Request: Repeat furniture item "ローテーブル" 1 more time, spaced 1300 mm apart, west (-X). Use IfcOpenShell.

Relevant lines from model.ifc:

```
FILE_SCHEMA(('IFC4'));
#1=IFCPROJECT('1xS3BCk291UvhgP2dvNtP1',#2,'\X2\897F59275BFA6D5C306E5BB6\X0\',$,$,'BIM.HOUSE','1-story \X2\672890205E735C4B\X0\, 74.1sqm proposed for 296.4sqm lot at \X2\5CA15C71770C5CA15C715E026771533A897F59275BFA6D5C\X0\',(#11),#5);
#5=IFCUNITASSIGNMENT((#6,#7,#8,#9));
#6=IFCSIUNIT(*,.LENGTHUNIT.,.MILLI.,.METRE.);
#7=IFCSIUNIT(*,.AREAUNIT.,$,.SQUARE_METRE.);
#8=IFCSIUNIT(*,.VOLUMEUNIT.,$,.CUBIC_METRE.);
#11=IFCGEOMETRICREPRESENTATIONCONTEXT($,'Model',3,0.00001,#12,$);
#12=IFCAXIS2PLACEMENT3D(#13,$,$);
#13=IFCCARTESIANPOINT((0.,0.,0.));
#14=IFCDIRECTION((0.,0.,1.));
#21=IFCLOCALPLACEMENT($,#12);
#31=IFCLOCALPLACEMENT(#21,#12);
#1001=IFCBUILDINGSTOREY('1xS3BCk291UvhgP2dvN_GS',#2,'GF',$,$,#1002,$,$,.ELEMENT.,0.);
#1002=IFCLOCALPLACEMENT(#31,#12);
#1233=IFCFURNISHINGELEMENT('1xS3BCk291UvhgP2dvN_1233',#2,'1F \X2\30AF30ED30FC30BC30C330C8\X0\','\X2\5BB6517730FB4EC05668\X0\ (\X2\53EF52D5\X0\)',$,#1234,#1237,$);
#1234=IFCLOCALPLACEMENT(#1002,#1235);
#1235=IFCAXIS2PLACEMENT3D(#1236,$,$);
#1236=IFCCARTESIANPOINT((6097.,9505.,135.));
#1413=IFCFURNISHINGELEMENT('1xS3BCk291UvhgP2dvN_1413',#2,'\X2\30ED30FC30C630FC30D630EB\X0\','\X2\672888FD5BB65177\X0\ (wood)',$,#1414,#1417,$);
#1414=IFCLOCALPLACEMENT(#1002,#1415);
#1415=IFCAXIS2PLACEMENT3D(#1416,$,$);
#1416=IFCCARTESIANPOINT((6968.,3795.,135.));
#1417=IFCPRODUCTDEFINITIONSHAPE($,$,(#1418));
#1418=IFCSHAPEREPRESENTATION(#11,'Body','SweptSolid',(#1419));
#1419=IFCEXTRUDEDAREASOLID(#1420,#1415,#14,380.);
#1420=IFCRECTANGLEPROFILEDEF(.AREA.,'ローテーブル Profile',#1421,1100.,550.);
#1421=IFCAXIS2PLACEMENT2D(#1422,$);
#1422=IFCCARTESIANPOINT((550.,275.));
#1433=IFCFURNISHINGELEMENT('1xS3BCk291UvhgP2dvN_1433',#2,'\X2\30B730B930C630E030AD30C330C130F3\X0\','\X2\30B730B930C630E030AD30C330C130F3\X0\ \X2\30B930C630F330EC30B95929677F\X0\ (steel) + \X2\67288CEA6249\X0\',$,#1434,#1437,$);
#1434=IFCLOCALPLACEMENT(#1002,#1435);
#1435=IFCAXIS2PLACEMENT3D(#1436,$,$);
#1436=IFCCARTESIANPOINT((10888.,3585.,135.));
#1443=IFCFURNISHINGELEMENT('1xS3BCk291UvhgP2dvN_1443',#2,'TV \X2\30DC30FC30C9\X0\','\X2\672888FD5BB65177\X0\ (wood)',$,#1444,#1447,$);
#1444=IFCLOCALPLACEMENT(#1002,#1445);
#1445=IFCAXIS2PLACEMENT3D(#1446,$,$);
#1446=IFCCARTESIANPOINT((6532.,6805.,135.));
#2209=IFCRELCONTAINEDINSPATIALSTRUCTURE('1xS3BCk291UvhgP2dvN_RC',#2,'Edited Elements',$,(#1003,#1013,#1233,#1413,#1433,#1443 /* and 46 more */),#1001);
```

```python
import numpy as np
import ifcopenshell
import ifcopenshell.api.geometry
import ifcopenshell.api.root
import ifcopenshell.util.element
import ifcopenshell.util.placement

model = ifcopenshell.open("model.ifc")


def reuse_history(source, copy):
    """copy_class also copies each property set's owner history, people and application; keep the originals."""
    for rel in copy.IsDefinedBy:
        if rel.is_a("IfcRelDefinesByProperties") and (history := rel.RelatingPropertyDefinition.OwnerHistory):
            rel.RelatingPropertyDefinition.OwnerHistory = source.OwnerHistory
            ifcopenshell.util.element.remove_deep2(model, history)


source = model.by_guid("1xS3BCk291UvhgP2dvN_1413")
base = ifcopenshell.util.placement.get_local_placement(source.ObjectPlacement)
step = np.array([-1.0, 0.0, 0.0]) * 1300.0

for i in range(1, 2):
    copy = ifcopenshell.api.root.copy_class(model, product=source)
    copy.Representation = ifcopenshell.util.element.copy_deep(
        model, source.Representation, exclude=["IfcGeometricRepresentationContext", "IfcRepresentationMap"]
    )
    reuse_history(source, copy)
    matrix = base.copy()
    matrix[:3, 3] += i * step
    print("added at", matrix[:3, 3].round(3) + 0.0)
    ifcopenshell.api.geometry.edit_object_placement(model, product=copy, matrix=matrix, is_si=False)

model.write("model_updated.ifc")
```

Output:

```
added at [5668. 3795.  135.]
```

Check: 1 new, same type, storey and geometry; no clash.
